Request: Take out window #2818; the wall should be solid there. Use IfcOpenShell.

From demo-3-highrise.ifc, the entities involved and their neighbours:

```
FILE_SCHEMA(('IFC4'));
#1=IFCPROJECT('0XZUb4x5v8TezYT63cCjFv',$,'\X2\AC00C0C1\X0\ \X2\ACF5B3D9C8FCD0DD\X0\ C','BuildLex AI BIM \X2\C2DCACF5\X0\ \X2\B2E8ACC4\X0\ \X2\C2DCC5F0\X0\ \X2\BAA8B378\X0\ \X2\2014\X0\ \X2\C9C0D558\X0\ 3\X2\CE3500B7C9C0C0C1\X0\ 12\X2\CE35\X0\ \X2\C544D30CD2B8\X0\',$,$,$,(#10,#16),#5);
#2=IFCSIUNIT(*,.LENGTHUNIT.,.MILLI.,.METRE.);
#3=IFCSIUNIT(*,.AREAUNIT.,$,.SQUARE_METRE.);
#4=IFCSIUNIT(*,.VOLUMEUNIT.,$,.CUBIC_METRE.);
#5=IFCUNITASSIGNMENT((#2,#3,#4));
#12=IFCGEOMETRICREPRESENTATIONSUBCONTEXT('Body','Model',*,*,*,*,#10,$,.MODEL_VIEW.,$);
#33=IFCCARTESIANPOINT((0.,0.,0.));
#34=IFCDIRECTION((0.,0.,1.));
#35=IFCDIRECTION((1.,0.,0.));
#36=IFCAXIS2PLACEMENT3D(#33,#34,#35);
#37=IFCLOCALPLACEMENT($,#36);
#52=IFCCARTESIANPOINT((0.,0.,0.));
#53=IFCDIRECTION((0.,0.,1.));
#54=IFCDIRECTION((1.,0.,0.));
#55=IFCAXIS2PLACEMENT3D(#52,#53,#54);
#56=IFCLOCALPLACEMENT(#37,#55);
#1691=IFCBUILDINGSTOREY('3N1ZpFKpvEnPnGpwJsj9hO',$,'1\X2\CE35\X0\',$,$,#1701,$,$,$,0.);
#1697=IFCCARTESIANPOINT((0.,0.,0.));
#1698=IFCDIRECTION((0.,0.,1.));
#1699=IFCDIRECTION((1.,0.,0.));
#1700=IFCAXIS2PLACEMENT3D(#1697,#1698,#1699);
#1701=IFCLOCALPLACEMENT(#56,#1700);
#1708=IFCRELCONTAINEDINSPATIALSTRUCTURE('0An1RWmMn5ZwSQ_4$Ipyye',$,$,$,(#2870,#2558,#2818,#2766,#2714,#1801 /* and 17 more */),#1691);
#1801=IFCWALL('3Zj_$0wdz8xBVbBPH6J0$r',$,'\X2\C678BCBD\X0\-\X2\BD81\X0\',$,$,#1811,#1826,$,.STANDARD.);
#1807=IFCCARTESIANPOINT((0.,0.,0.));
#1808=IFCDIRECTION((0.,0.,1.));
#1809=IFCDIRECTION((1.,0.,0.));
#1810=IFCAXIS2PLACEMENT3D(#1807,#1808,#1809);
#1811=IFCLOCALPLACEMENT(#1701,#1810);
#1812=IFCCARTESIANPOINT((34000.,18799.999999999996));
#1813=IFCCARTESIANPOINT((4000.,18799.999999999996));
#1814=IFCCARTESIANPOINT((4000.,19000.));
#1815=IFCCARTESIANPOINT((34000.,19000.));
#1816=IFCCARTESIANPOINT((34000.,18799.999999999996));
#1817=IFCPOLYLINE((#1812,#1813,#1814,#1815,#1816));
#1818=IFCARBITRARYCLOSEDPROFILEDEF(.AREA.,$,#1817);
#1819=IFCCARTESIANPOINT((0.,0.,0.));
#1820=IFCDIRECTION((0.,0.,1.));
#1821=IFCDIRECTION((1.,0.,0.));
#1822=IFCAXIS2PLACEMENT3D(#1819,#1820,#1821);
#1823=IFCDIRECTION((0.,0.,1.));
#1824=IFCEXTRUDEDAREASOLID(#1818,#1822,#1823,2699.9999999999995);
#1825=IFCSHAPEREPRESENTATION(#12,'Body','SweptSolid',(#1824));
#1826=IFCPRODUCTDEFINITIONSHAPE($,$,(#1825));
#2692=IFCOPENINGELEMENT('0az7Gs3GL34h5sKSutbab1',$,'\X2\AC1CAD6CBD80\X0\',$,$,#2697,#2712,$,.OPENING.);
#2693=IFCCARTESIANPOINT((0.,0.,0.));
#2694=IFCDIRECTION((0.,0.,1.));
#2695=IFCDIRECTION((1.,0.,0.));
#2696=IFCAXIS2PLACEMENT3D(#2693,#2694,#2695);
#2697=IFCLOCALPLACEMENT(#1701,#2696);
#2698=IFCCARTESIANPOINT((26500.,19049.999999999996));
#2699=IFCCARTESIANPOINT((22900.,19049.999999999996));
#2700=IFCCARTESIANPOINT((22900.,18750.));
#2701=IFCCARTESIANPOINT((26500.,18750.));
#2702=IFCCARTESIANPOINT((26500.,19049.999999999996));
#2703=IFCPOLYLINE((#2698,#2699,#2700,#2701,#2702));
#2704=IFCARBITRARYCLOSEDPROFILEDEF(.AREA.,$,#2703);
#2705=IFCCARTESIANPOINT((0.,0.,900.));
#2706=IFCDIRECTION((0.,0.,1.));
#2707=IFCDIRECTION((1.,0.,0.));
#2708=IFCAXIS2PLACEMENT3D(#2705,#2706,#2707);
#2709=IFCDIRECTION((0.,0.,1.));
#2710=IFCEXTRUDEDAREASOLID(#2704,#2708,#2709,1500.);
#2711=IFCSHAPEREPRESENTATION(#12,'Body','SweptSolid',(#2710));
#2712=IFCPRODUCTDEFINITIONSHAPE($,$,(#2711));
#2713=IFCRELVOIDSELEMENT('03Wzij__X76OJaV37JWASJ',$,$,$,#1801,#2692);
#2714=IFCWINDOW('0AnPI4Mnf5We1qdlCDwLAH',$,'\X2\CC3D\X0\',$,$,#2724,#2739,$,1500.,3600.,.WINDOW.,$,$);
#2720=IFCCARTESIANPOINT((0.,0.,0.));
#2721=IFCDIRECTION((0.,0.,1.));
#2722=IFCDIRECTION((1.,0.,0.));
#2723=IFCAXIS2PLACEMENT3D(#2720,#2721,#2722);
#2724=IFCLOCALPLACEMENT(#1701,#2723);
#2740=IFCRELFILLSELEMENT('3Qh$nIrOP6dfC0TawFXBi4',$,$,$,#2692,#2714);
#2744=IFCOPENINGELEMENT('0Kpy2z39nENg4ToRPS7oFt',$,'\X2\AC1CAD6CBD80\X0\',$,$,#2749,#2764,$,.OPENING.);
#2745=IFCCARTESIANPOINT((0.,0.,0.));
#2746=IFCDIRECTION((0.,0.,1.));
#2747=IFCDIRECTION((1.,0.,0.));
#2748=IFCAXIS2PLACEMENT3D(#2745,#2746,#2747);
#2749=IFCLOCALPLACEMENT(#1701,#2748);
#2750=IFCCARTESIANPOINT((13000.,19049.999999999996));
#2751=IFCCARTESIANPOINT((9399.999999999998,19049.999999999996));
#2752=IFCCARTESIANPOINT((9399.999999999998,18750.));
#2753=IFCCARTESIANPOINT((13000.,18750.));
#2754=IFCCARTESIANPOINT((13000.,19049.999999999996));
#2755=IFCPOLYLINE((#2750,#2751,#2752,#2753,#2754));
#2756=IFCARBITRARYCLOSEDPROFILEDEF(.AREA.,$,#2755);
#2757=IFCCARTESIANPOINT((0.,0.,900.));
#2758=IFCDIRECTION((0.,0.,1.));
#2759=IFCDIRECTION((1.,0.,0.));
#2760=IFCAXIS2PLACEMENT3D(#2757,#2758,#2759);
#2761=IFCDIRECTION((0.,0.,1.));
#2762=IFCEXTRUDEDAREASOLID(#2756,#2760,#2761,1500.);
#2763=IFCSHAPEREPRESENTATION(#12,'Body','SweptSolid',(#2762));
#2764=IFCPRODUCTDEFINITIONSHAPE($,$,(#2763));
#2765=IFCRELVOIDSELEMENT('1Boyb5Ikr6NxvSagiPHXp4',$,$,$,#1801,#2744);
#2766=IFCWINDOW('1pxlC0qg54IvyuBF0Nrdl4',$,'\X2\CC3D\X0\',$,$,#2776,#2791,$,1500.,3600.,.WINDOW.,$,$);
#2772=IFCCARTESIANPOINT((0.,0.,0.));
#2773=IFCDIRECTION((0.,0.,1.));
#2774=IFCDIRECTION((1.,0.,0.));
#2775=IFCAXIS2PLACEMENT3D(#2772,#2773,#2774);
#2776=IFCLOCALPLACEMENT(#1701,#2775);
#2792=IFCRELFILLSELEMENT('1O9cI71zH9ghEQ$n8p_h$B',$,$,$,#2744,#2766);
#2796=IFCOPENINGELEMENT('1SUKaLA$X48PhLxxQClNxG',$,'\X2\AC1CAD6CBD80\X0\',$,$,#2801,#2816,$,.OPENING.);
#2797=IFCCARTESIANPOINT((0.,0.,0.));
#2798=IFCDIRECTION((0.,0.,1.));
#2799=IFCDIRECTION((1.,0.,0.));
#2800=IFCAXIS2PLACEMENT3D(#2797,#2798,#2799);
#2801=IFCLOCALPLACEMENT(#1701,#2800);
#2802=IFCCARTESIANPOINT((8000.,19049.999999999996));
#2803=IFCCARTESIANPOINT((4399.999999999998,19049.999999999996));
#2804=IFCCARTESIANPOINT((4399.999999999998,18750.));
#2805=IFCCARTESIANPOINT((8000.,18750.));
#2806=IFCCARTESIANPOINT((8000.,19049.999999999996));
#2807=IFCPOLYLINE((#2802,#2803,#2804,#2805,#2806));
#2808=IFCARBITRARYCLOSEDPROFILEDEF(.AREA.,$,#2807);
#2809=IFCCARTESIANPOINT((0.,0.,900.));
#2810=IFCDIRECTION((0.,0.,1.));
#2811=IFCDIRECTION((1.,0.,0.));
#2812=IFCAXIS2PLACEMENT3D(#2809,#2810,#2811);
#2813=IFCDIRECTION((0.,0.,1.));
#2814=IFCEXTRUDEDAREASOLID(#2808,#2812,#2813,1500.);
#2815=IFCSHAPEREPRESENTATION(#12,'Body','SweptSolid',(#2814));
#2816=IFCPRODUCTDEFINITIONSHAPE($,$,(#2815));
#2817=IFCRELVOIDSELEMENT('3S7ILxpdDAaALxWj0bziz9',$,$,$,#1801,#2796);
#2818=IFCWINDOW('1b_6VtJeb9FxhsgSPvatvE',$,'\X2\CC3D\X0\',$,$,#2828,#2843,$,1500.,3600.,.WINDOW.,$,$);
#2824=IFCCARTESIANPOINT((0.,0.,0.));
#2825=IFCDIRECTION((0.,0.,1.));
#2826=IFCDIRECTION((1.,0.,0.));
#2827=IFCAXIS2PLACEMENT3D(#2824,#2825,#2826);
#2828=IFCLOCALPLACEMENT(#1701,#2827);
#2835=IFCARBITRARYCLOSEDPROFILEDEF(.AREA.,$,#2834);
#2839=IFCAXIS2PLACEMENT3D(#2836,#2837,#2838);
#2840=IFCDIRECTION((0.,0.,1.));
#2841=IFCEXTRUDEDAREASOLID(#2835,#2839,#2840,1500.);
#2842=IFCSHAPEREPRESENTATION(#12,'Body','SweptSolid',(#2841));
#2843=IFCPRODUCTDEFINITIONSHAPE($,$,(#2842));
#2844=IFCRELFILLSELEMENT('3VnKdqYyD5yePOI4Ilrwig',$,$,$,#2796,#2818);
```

```python
import ifcopenshell
import ifcopenshell.api.feature
import ifcopenshell.api.root
import ifcopenshell.geom
import ifcopenshell.util.shape

model = ifcopenshell.open("demo-3-highrise.ifc")
settings = ifcopenshell.geom.settings()


def volume(element):
    """Net volume in cubic metres, openings subtracted."""
    shape = ifcopenshell.geom.create_shape(settings, element)
    return ifcopenshell.util.shape.get_volume(shape.geometry)


window = model.by_guid("1b_6VtJeb9FxhsgSPvatvE")
opening = window.FillsVoids[0].RelatingOpeningElement
wall = opening.VoidsElements[0].RelatingBuildingElement
before = volume(wall)

ifcopenshell.api.root.remove_product(model, product=window)
ifcopenshell.api.feature.remove_feature(model, feature=opening)

after = volume(wall)

print(f"wall volume {before:.3f} -> {after:.3f} m3")

model.write("demo-3-highrise_v2.ifc")
```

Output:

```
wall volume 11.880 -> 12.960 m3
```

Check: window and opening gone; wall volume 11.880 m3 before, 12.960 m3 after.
